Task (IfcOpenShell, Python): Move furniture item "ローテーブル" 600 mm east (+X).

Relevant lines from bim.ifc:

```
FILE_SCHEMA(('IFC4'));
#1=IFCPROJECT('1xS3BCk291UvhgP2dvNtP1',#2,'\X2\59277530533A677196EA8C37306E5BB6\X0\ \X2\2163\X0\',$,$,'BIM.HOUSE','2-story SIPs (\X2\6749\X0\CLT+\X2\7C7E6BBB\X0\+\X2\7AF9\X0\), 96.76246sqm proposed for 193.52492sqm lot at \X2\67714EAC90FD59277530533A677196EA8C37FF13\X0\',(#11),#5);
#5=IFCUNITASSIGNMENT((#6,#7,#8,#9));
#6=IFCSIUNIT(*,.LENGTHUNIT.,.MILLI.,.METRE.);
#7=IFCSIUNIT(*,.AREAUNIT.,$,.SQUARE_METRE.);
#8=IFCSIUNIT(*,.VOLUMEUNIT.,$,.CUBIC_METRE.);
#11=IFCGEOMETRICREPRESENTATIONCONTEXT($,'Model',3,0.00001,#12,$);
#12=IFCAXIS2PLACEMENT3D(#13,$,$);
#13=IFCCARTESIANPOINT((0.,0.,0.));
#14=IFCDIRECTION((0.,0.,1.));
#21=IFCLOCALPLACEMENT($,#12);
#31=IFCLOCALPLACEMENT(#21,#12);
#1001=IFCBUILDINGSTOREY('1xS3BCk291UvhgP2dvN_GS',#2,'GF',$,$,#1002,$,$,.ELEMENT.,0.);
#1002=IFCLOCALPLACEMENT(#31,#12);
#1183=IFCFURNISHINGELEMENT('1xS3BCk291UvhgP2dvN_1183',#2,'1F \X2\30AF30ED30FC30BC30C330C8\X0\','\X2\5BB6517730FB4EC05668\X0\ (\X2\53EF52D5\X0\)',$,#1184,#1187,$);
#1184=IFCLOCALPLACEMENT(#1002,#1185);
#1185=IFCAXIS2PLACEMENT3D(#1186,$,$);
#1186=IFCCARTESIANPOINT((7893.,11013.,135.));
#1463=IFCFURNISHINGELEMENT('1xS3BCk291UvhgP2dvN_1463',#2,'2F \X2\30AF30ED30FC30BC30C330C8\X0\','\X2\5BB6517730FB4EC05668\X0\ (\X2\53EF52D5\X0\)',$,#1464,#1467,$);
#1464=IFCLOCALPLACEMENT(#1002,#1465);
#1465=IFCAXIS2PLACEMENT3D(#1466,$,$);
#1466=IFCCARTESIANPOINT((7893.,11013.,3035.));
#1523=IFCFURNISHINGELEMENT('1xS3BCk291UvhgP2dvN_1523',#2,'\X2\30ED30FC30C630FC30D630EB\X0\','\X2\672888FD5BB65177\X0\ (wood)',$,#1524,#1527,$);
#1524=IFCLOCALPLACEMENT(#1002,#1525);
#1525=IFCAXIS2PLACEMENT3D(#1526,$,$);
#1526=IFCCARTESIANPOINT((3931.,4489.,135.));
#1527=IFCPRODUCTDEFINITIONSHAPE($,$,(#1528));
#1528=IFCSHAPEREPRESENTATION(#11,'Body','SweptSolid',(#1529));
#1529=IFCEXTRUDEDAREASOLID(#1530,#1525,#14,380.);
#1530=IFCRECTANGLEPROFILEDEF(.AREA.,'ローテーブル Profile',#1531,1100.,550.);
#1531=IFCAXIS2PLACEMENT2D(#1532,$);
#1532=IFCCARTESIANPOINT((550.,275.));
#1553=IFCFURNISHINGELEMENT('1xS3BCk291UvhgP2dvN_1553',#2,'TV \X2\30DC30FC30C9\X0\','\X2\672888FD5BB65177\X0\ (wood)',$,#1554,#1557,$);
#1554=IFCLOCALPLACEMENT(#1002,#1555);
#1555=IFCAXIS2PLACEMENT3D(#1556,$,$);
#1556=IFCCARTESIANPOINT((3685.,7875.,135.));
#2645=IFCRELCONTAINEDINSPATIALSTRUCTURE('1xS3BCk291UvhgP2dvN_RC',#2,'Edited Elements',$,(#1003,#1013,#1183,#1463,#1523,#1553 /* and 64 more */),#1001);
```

```python
import ifcopenshell
import ifcopenshell.api.geometry
import ifcopenshell.util.placement
import ifcopenshell.util.unit

model = ifcopenshell.open("bim.ifc")
unit_scale = ifcopenshell.util.unit.calculate_unit_scale(model)

item = model.by_guid("1xS3BCk291UvhgP2dvN_1523")
matrix = ifcopenshell.util.placement.get_local_placement(item.ObjectPlacement)
matrix[0, 3] += 0.6 / unit_scale
ifcopenshell.api.geometry.edit_object_placement(model, product=item, matrix=matrix, is_si=False)

print(ifcopenshell.util.placement.get_local_placement(item.ObjectPlacement).round(3) + 0.0)

model.write("bim_rev.ifc")
```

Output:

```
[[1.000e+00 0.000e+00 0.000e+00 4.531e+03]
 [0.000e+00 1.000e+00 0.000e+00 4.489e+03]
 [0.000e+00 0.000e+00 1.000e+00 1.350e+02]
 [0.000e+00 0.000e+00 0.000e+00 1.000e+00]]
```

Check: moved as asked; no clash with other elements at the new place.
